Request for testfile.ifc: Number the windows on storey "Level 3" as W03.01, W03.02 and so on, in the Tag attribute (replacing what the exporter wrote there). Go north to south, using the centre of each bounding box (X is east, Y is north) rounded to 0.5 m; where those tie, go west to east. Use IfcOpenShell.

First a look at what the model holds.

```python
import ifcopenshell
import ifcopenshell.util.element
import ifcopenshell.util.placement

model = ifcopenshell.open("testfile.ifc")
print(model.schema)
storey = next(s for s in model.by_type("IfcBuildingStorey") if s.Name == "Level 3")
windows = [e for e in ifcopenshell.util.element.get_decomposition(storey) if e.is_a("IfcWindow")]
for e in sorted(windows, key=lambda e: e.id()):
    origin = ifcopenshell.util.placement.get_local_placement(e.ObjectPlacement)[:3, 3]
    print(e.id(), e.Tag, e.Name, origin.round(2) + 0.0, sep=" | ")
```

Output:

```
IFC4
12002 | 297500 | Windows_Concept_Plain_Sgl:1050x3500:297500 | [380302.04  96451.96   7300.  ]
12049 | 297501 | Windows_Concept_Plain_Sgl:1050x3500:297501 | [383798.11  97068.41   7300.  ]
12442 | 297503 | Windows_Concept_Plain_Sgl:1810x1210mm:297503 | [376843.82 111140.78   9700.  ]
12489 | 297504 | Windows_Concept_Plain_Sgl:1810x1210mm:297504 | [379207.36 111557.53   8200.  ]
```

```python
import ifcopenshell
import ifcopenshell.geom
import ifcopenshell.util.element
import ifcopenshell.util.shape

model = ifcopenshell.open("testfile.ifc")
settings = ifcopenshell.geom.settings()
settings.set("use-world-coords", True)


def centre(element):
    shape = ifcopenshell.geom.create_shape(settings, element)
    return ifcopenshell.util.shape.get_bbox_centroid(shape.geometry)


storey = next(s for s in model.by_type("IfcBuildingStorey") if s.Name == "Level 3")
windows = [e for e in ifcopenshell.util.element.get_decomposition(storey) if e.is_a("IfcWindow")]

# Insertion points can sit at a corner or the storey origin, so sort by the geometry (in metres).
centres = {e: centre(e) for e in windows}
windows.sort(key=lambda e: (-round(centres[e][1] / 0.5), centres[e][0]))

for i, e in enumerate(windows, start=1):
    number = f"W03.{i:02d}"
    e.Tag = number
    print(e.id(), number)

model.write("testfile-out.ifc")
```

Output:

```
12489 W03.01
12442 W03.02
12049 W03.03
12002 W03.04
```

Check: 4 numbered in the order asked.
